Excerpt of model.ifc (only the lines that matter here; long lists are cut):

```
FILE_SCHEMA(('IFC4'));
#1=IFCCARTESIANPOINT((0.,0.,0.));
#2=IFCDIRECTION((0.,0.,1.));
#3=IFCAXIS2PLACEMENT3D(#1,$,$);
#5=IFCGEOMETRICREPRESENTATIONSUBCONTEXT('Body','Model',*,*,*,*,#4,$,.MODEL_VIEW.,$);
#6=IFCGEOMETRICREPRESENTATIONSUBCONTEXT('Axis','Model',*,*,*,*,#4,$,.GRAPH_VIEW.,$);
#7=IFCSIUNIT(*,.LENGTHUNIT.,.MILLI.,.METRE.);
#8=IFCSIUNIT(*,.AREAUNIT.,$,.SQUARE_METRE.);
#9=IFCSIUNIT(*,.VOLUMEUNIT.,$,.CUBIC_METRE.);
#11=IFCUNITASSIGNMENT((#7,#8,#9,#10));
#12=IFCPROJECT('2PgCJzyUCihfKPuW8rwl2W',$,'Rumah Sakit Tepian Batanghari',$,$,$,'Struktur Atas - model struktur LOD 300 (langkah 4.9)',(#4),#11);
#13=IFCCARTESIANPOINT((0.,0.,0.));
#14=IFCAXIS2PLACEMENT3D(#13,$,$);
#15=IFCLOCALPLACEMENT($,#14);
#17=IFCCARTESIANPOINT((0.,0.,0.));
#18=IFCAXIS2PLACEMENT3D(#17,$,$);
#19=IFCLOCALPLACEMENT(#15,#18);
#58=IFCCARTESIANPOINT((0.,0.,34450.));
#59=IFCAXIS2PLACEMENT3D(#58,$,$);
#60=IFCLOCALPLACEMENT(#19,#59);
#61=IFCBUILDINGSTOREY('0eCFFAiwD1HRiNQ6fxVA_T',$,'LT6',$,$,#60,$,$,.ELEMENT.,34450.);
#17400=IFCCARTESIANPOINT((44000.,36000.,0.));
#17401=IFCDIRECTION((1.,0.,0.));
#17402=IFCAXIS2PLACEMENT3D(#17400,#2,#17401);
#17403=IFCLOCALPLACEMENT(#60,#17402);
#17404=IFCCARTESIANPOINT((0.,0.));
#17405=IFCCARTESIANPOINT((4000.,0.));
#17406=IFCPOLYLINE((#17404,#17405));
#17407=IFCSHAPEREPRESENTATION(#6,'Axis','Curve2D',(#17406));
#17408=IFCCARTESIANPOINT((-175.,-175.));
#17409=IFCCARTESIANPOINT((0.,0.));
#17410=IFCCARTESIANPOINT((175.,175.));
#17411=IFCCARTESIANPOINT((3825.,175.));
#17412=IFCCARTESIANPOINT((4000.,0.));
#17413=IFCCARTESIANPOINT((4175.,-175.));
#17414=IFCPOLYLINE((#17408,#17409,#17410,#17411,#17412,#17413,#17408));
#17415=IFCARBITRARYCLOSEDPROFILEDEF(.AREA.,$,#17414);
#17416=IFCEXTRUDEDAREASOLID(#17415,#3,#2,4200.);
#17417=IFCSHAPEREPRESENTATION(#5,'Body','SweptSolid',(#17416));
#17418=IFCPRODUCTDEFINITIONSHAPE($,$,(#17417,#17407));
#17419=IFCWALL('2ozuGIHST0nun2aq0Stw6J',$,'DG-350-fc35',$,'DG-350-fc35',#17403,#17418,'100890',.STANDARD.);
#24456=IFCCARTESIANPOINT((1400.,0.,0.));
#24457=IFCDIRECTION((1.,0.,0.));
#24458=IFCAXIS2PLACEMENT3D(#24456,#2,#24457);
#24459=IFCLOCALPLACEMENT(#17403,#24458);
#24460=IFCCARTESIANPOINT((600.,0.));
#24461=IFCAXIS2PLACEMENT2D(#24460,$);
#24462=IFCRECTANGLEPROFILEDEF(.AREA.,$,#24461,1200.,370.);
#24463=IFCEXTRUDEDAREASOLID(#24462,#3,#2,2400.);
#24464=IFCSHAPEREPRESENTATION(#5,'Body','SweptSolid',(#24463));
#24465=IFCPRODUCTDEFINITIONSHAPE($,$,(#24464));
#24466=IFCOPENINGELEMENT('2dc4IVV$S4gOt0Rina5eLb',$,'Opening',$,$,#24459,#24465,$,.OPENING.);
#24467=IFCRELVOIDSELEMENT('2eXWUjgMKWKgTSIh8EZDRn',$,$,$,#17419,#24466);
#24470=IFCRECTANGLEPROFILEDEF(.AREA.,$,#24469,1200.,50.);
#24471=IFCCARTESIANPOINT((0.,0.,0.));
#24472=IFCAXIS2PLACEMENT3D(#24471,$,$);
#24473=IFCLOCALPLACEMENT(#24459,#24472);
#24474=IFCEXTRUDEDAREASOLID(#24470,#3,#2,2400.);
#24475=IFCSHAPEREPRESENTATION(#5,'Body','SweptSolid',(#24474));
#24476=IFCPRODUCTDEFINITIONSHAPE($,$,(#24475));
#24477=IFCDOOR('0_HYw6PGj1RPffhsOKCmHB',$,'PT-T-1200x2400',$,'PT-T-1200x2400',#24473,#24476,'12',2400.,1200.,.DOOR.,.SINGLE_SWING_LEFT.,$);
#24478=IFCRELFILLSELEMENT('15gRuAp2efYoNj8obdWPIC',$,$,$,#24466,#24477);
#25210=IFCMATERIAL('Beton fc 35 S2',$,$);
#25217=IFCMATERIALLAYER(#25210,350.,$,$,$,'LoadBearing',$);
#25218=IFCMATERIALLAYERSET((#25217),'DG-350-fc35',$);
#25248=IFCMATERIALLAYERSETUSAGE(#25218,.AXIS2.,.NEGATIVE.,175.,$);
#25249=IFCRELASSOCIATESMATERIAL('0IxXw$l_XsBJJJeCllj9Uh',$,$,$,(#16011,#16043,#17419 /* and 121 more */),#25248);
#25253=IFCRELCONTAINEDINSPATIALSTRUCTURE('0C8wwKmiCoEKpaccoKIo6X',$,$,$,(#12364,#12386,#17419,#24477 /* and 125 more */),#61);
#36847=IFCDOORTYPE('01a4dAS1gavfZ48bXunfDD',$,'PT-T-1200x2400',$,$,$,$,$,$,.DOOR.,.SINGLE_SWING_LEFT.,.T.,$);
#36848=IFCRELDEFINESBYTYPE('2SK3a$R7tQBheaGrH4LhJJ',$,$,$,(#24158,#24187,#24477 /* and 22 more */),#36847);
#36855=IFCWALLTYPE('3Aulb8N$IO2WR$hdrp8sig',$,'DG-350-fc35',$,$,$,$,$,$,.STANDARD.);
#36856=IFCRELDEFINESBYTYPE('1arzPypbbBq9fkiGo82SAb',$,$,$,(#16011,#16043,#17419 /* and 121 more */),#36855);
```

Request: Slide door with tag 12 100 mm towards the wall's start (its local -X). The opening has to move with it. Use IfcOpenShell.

```python
import ifcopenshell
import ifcopenshell.api.geometry
import ifcopenshell.util.placement
import ifcopenshell.util.unit

model = ifcopenshell.open("model.ifc")
unit_scale = ifcopenshell.util.unit.calculate_unit_scale(model)

door = model.by_guid("0_HYw6PGj1RPffhsOKCmHB")
opening = door.FillsVoids[0].RelatingOpeningElement
wall = opening.VoidsElements[0].RelatingBuildingElement

wall_matrix = ifcopenshell.util.placement.get_local_placement(wall.ObjectPlacement)
shift = wall_matrix[:3, 0] * -0.1 / unit_scale
before = ifcopenshell.util.placement.get_local_placement(door.ObjectPlacement)[:3, 3].copy()

# The door is placed relative to its opening, so it follows when the opening moves.
matrix = ifcopenshell.util.placement.get_local_placement(opening.ObjectPlacement)
matrix[:3, 3] += shift
ifcopenshell.api.geometry.edit_object_placement(
    model, product=opening, matrix=matrix, is_si=False, should_transform_children=True
)

after = ifcopenshell.util.placement.get_local_placement(door.ObjectPlacement)[:3, 3]
print("door moved by", (after - before).round(3) + 0.0)

model.write("model_edited.ifc")
```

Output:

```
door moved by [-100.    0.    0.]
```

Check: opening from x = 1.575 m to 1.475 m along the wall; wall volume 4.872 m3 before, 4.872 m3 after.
